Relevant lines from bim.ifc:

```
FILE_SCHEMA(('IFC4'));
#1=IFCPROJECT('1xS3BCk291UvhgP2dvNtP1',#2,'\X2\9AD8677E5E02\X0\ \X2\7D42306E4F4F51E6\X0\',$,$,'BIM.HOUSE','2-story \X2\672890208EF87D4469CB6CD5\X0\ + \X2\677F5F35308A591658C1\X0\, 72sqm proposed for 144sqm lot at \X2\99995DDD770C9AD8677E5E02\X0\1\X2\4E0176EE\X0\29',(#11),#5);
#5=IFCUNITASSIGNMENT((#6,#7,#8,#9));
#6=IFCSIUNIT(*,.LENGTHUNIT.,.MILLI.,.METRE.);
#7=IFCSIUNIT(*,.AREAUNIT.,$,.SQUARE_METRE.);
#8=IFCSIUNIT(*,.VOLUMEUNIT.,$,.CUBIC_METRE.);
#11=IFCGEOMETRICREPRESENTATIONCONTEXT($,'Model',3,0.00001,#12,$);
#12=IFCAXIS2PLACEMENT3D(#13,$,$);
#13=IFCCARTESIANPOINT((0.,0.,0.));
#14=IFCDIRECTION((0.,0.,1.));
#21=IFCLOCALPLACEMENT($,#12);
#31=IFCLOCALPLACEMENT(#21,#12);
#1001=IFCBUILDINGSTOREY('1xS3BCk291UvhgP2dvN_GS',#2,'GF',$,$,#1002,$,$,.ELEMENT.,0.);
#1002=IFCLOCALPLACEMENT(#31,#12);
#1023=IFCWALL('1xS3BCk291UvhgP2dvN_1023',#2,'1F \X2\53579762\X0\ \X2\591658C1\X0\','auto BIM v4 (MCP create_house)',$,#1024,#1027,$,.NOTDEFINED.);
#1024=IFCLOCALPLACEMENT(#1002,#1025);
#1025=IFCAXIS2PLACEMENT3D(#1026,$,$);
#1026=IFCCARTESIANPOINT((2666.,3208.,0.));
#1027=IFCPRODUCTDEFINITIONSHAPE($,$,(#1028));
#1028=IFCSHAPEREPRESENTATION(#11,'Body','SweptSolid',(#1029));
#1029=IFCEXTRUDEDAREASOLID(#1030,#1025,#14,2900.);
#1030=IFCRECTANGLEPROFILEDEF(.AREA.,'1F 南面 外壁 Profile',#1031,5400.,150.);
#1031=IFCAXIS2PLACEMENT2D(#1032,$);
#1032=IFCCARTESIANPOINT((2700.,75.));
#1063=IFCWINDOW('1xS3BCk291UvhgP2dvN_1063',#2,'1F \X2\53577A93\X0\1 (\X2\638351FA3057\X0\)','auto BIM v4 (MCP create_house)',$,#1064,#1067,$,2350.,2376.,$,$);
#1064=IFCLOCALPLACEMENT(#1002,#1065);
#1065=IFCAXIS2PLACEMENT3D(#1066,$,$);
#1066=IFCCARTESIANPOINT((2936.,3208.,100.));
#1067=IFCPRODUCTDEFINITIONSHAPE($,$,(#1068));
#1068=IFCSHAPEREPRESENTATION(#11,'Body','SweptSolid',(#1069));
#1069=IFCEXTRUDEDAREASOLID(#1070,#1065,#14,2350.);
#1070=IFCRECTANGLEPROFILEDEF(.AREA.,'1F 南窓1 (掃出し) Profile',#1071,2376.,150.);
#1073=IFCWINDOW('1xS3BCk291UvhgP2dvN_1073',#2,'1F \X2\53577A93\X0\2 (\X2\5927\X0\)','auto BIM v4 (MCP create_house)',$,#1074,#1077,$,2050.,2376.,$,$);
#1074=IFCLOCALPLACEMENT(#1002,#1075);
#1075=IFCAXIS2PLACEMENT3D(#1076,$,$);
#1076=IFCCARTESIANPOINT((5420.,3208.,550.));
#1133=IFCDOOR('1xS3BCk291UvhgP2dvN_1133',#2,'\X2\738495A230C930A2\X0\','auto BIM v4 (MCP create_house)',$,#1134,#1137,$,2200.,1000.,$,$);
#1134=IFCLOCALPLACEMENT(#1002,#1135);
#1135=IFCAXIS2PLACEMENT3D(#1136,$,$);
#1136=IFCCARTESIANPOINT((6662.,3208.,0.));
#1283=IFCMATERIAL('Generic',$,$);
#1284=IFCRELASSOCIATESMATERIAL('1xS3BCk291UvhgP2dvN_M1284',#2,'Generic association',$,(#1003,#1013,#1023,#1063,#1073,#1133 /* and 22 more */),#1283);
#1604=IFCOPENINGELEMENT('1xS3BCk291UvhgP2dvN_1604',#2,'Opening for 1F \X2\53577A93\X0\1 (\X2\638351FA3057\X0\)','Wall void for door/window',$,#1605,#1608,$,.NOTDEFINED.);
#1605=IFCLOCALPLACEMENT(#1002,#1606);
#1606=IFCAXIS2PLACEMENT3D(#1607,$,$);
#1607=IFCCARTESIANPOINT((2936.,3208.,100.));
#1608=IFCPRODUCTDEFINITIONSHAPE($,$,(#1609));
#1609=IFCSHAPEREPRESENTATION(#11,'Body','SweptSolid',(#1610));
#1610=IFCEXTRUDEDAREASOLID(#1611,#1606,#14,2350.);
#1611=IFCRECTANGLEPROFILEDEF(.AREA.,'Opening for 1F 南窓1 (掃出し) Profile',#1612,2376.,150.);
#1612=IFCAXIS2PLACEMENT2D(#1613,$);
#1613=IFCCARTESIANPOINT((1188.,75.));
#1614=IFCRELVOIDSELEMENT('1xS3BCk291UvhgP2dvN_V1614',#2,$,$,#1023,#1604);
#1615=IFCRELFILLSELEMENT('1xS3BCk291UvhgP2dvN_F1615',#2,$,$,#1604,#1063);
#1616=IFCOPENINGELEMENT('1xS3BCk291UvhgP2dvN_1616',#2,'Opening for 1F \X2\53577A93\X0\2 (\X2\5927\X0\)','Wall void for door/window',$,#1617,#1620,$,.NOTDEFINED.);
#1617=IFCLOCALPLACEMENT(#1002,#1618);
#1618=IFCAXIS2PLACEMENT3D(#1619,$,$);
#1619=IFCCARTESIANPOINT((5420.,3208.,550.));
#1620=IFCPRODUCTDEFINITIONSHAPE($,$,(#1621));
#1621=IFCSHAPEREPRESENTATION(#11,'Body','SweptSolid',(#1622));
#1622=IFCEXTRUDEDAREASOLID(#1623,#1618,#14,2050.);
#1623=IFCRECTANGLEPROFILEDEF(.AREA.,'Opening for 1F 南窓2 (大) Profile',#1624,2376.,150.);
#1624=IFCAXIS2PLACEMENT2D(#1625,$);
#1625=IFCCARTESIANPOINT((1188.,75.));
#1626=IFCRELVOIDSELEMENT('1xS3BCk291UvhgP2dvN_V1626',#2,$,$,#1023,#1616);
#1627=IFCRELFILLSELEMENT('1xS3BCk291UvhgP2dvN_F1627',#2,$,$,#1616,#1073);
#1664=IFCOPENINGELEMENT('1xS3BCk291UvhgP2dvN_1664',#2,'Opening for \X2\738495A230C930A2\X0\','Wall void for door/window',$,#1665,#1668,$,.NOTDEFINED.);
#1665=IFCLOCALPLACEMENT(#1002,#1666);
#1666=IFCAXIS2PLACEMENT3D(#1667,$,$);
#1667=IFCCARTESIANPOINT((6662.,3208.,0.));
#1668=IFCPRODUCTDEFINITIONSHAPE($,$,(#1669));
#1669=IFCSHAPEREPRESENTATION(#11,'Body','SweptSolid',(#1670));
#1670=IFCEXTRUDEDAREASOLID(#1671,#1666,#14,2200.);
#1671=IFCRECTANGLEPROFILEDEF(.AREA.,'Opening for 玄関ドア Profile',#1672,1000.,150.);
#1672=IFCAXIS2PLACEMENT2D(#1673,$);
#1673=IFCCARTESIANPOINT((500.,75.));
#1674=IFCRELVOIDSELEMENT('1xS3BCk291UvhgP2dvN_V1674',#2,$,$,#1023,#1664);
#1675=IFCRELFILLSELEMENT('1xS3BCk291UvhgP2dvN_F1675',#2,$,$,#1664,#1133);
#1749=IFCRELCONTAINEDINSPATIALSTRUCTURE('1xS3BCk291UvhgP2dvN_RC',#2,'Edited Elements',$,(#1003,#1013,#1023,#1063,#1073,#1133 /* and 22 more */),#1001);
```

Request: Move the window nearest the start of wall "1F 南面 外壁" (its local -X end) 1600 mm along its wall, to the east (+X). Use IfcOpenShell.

```python
import ifcopenshell
import ifcopenshell.api.geometry
import ifcopenshell.util.placement
import ifcopenshell.util.unit

model = ifcopenshell.open("bim.ifc")
unit_scale = ifcopenshell.util.unit.calculate_unit_scale(model)

window = model.by_guid("1xS3BCk291UvhgP2dvN_1063")
opening = window.FillsVoids[0].RelatingOpeningElement
wall = opening.VoidsElements[0].RelatingBuildingElement

wall_matrix = ifcopenshell.util.placement.get_local_placement(wall.ObjectPlacement)
shift = wall_matrix[:3, 0] * 1.6 / unit_scale
before = ifcopenshell.util.placement.get_local_placement(window.ObjectPlacement)[:3, 3].copy()

# The window is not placed relative to its opening, so move both.
for product in (opening, window):
    matrix = ifcopenshell.util.placement.get_local_placement(product.ObjectPlacement)
    matrix[:3, 3] += shift
    ifcopenshell.api.geometry.edit_object_placement(model, product=product, matrix=matrix, is_si=False)

after = ifcopenshell.util.placement.get_local_placement(window.ObjectPlacement)[:3, 3]
print("window moved by", (after - before).round(3) + 0.0)

model.write("bim_v2.ifc")
```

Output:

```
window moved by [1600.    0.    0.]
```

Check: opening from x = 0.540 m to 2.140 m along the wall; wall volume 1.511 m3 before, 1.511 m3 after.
